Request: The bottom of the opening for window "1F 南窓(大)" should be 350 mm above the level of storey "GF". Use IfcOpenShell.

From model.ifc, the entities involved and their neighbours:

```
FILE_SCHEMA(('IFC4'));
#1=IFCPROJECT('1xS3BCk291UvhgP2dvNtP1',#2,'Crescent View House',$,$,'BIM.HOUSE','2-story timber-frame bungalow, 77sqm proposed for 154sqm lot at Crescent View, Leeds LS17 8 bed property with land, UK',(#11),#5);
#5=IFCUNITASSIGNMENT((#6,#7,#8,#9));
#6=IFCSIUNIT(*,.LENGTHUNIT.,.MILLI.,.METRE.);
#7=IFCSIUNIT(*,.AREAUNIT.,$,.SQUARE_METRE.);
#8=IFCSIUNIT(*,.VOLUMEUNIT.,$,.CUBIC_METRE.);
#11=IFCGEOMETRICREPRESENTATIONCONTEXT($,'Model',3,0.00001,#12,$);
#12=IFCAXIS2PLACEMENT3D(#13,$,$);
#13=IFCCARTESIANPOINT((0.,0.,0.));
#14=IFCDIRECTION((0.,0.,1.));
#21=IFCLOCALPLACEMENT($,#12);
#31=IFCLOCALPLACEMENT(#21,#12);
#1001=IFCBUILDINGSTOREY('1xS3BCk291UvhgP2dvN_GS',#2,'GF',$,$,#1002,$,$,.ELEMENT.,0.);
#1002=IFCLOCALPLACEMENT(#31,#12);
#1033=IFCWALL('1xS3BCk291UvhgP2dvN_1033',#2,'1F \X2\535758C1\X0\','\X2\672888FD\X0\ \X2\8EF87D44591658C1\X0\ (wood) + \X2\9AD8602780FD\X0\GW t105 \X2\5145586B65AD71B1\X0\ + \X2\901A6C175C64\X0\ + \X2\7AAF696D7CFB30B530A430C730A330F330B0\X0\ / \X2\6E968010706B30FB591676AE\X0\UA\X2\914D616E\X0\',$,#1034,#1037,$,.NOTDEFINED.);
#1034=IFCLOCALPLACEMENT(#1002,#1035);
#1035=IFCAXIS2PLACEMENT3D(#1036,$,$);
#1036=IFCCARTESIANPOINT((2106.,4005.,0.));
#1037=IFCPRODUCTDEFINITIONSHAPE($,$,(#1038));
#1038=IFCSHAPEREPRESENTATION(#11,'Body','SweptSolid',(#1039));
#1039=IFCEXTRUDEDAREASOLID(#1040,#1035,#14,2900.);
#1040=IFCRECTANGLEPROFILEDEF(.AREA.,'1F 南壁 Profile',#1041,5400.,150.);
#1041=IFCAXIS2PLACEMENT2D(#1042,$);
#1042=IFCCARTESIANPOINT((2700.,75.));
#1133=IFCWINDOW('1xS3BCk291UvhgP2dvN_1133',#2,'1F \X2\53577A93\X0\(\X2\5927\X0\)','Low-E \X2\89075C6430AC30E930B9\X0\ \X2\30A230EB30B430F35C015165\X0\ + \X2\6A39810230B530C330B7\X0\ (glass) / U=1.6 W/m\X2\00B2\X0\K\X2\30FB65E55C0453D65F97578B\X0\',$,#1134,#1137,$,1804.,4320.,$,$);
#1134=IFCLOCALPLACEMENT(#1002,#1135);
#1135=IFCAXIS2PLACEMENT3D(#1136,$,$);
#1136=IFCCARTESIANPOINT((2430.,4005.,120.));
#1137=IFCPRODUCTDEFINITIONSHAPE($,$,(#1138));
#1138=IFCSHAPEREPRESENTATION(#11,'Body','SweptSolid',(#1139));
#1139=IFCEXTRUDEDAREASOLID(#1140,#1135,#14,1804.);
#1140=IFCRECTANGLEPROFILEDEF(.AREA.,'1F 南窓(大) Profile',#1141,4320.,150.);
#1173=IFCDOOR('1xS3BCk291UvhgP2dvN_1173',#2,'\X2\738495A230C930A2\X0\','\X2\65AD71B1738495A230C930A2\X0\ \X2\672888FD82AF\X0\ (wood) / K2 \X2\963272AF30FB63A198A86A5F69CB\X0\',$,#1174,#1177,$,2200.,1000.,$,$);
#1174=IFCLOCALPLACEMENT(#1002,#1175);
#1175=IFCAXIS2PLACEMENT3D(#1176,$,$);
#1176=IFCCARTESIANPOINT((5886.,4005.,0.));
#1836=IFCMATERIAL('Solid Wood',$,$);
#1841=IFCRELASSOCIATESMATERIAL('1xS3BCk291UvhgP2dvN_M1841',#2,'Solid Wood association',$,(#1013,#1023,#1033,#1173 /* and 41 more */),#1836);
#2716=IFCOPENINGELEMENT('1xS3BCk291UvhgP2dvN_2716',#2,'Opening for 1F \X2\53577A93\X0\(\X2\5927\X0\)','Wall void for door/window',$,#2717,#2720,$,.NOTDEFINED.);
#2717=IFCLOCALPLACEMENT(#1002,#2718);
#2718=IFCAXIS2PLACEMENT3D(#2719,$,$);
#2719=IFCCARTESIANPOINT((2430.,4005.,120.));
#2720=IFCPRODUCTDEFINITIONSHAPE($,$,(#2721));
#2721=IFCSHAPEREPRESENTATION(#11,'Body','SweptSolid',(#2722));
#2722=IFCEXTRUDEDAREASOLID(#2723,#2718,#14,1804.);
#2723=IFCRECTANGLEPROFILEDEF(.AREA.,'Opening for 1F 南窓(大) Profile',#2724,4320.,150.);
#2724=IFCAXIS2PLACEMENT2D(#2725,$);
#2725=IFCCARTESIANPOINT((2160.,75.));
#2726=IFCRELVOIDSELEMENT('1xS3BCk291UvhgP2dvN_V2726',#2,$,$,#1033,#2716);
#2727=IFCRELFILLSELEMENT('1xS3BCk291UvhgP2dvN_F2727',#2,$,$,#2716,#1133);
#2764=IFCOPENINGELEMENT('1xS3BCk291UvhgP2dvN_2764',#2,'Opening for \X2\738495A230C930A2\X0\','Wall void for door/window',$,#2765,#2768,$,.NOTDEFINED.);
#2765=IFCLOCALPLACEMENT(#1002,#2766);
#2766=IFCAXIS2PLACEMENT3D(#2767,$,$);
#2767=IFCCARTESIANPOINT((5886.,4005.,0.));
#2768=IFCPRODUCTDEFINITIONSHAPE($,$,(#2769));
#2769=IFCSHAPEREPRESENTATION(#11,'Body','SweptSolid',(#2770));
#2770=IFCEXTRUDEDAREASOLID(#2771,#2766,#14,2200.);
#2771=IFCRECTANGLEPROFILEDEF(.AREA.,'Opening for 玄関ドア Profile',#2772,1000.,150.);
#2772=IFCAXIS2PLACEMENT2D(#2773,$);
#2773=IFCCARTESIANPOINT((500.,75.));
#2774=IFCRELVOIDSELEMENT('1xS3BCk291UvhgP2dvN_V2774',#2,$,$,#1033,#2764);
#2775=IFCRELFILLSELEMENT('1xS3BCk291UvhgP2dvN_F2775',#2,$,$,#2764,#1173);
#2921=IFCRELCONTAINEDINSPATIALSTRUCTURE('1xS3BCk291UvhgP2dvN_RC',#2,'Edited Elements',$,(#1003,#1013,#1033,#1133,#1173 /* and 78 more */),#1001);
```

```python
import numpy as np
import ifcopenshell
import ifcopenshell.api.geometry
import ifcopenshell.geom
import ifcopenshell.util.element
import ifcopenshell.util.placement
import ifcopenshell.util.shape
import ifcopenshell.util.unit

model = ifcopenshell.open("model.ifc")
unit_scale = ifcopenshell.util.unit.calculate_unit_scale(model)

window = model.by_guid("1xS3BCk291UvhgP2dvN_1133")
opening = window.FillsVoids[0].RelatingOpeningElement
storey = ifcopenshell.util.element.get_container(window, ifc_class="IfcBuildingStorey")
level = ifcopenshell.util.placement.get_local_placement(storey.ObjectPlacement)[2, 3]

# The opening's origin need not be at the sill, so measure its lowest point.
shape = ifcopenshell.geom.create_shape(ifcopenshell.geom.settings(), opening)
bottom = ifcopenshell.util.shape.get_shape_bottom_elevation(shape, shape.geometry) / unit_scale
dz = level + 350.0 - bottom

shift = np.array([0.0, 0.0, dz])
# The window is not placed relative to its opening, so move both.
for product in (opening, window):
    matrix = ifcopenshell.util.placement.get_local_placement(product.ObjectPlacement)
    matrix[:3, 3] += shift
    ifcopenshell.api.geometry.edit_object_placement(model, product=product, matrix=matrix, is_si=False)

print(f"moved by {dz * unit_scale:+.3f} m")

model.write("model_edited.ifc")
```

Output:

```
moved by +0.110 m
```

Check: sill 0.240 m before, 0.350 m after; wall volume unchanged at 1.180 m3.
